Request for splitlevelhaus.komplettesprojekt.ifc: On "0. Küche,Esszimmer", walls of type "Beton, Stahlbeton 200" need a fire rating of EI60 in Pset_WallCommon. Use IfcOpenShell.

First a look at what the model holds.

```python
import ifcopenshell
import ifcopenshell.util.element

model = ifcopenshell.open("splitlevelhaus.komplettesprojekt.ifc")
print(model.schema)
storey = next(s for s in model.by_type("IfcBuildingStorey") if s.Name == "0. Küche,Esszimmer")
walls = [e for e in ifcopenshell.util.element.get_decomposition(storey) if e.is_a("IfcWall")]
seen = {}
for e in walls:
    element_type = ifcopenshell.util.element.get_type(e)
    key = (element_type.Name if element_type != e and element_type else None, ifcopenshell.util.element.get_pset(e, "Pset_WallCommon", "FireRating"))
    seen[key] = seen.get(key, 0) + 1
for (name, value), count in sorted(seen.items(), key=str):
    print(count, "x", name, "|", value)
```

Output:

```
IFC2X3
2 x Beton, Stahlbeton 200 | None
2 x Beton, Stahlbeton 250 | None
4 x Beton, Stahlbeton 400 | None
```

```python
import ifcopenshell
import ifcopenshell.api.pset
import ifcopenshell.util.element

model = ifcopenshell.open("splitlevelhaus.komplettesprojekt.ifc")

storey = next(s for s in model.by_type("IfcBuildingStorey") if s.Name == "0. Küche,Esszimmer")
walls = [e for e in ifcopenshell.util.element.get_decomposition(storey) if e.is_a("IfcWall")]

count = 0
for e in walls:
    element_type = ifcopenshell.util.element.get_type(e)
    if element_type in (None, e) or element_type.Name != "Beton, Stahlbeton 200":
        continue
    # add_pset returns the element's existing set when there is one.
    pset = ifcopenshell.api.pset.add_pset(model, product=e, name="Pset_WallCommon")
    ifcopenshell.api.pset.edit_pset(model, pset=pset, properties={"FireRating": "EI60"})
    count += 1

print(count, "walls updated")

model.write("splitlevelhaus.komplettesprojekt_rev.ifc")
```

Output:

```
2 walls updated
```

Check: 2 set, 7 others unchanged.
